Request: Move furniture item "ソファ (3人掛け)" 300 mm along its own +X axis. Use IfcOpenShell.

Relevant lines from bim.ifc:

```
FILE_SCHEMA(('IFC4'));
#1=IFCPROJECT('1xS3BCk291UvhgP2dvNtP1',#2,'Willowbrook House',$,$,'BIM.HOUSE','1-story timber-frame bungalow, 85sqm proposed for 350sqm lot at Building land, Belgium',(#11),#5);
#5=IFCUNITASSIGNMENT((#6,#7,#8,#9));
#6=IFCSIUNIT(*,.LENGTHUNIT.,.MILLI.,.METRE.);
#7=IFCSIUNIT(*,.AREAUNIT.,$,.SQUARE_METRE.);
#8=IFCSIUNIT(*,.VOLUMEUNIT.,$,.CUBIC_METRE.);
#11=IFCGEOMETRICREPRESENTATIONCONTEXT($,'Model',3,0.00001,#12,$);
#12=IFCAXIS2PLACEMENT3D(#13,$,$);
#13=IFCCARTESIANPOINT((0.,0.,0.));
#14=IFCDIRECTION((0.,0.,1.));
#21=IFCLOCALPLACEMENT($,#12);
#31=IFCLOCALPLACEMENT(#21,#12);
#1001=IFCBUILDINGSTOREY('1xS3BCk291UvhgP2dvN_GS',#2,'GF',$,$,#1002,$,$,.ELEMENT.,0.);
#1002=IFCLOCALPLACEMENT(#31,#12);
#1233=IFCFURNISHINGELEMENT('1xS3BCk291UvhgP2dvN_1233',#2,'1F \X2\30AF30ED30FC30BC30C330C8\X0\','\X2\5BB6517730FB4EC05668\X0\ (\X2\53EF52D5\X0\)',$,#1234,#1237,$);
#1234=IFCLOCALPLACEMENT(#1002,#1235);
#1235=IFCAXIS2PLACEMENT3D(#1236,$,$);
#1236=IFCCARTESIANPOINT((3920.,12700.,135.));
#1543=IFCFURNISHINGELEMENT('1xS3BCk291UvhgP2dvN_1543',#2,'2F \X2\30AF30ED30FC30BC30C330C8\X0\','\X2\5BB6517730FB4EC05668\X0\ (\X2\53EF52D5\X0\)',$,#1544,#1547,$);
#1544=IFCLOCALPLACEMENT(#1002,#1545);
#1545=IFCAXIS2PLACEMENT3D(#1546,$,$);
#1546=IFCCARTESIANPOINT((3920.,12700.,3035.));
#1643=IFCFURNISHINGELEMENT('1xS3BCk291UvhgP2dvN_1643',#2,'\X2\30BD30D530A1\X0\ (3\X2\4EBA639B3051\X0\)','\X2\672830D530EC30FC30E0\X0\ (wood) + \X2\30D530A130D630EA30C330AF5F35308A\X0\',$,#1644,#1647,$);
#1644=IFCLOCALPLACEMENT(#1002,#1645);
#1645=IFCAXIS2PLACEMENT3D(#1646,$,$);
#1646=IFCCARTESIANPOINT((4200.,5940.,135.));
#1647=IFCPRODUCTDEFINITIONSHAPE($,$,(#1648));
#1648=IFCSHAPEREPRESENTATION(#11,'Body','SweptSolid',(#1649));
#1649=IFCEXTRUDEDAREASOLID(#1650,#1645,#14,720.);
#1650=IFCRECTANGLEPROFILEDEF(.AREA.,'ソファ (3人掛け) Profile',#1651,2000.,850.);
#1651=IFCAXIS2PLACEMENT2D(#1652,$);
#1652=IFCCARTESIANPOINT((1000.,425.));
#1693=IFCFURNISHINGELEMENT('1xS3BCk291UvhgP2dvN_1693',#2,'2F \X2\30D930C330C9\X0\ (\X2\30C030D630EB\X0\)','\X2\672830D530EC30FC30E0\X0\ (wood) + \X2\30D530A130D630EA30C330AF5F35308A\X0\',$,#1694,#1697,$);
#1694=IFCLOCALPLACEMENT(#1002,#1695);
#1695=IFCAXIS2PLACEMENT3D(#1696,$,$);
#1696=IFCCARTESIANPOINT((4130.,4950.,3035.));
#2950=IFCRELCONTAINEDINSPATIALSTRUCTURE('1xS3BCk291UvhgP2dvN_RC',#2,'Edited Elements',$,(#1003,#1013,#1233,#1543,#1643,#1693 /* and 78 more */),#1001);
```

```python
import ifcopenshell
import ifcopenshell.api.geometry
import ifcopenshell.util.placement
import ifcopenshell.util.unit

model = ifcopenshell.open("bim.ifc")
unit_scale = ifcopenshell.util.unit.calculate_unit_scale(model)

item = model.by_guid("1xS3BCk291UvhgP2dvN_1643")
matrix = ifcopenshell.util.placement.get_local_placement(item.ObjectPlacement)
matrix[:3, 3] += matrix[:3, 0] * 0.3 / unit_scale
ifcopenshell.api.geometry.edit_object_placement(model, product=item, matrix=matrix, is_si=False)

print(ifcopenshell.util.placement.get_local_placement(item.ObjectPlacement).round(3) + 0.0)

model.write("bim-out.ifc")
```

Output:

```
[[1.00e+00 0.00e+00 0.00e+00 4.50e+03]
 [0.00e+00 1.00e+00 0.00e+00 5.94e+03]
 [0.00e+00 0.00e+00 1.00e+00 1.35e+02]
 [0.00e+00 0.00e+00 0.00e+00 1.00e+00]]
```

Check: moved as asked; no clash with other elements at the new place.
